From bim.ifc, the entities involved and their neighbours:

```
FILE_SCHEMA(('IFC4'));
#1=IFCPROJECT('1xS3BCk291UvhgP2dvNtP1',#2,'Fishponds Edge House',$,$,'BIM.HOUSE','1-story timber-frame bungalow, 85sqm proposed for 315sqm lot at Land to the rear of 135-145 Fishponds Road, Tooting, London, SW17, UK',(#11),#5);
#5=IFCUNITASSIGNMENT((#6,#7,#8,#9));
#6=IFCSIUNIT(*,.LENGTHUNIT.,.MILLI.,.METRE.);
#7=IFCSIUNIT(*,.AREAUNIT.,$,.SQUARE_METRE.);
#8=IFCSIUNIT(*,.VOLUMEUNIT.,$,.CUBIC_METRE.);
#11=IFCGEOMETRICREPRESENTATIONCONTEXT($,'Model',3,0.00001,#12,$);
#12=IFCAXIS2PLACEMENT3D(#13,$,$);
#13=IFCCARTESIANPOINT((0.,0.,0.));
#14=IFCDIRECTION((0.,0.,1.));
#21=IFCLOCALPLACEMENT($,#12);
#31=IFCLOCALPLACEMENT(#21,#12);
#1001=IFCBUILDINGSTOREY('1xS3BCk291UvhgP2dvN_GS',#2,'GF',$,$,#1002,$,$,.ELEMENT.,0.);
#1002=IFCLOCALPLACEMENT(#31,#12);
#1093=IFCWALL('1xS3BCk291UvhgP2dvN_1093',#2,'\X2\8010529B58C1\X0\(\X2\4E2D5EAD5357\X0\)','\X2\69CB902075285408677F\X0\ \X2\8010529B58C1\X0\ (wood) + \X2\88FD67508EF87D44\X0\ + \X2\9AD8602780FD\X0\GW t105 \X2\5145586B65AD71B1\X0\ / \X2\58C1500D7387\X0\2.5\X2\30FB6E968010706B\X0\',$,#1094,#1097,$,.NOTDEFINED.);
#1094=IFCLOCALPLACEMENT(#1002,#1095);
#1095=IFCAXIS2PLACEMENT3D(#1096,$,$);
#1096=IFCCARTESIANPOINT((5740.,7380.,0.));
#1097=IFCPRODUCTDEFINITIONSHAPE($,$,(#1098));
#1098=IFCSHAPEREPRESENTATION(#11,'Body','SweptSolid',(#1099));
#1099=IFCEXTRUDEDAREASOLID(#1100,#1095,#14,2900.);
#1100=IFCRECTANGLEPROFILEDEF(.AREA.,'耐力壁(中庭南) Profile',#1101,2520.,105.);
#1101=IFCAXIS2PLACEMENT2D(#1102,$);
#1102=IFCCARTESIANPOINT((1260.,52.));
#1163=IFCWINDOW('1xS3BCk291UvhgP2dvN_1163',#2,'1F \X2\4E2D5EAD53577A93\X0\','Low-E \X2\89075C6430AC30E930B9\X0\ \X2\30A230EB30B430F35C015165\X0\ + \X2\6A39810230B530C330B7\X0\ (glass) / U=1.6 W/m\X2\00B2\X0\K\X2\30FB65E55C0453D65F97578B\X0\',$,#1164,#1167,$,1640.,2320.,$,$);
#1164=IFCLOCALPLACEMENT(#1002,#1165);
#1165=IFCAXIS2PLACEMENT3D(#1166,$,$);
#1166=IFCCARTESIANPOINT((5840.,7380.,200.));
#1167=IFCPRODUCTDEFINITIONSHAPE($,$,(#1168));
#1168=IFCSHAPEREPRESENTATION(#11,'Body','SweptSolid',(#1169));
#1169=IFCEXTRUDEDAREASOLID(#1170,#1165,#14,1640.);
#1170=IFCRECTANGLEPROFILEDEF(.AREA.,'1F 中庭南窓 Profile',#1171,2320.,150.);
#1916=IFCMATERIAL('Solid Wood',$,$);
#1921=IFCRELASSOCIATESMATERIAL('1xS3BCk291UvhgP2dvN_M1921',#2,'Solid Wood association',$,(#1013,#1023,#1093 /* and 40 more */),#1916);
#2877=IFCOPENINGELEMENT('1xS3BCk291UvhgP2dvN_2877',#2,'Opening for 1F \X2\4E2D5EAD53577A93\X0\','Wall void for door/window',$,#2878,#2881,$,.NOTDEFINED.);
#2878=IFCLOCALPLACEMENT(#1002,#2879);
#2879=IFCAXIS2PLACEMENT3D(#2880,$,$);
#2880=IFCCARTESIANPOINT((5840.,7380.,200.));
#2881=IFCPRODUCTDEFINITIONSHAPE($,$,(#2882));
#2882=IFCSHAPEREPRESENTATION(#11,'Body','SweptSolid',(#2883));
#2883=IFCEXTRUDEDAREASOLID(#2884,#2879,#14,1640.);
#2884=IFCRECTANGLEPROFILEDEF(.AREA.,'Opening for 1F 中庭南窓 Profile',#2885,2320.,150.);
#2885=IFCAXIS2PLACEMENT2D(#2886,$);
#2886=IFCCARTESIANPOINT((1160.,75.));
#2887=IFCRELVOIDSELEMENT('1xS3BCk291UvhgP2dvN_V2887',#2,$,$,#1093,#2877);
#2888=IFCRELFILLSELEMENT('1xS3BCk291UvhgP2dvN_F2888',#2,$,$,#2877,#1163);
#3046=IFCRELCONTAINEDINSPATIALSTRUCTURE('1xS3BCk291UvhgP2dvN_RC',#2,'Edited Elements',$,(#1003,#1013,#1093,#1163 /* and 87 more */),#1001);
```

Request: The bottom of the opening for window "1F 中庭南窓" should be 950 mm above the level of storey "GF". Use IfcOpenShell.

```python
import numpy as np
import ifcopenshell
import ifcopenshell.api.geometry
import ifcopenshell.geom
import ifcopenshell.util.element
import ifcopenshell.util.placement
import ifcopenshell.util.shape
import ifcopenshell.util.unit

model = ifcopenshell.open("bim.ifc")
unit_scale = ifcopenshell.util.unit.calculate_unit_scale(model)

window = model.by_guid("1xS3BCk291UvhgP2dvN_1163")
opening = window.FillsVoids[0].RelatingOpeningElement
storey = ifcopenshell.util.element.get_container(window, ifc_class="IfcBuildingStorey")
level = ifcopenshell.util.placement.get_local_placement(storey.ObjectPlacement)[2, 3]

# The opening's origin need not be at the sill, so measure its lowest point.
shape = ifcopenshell.geom.create_shape(ifcopenshell.geom.settings(), opening)
bottom = ifcopenshell.util.shape.get_shape_bottom_elevation(shape, shape.geometry) / unit_scale
dz = level + 950.0 - bottom

shift = np.array([0.0, 0.0, dz])
# The window is not placed relative to its opening, so move both.
for product in (opening, window):
    matrix = ifcopenshell.util.placement.get_local_placement(product.ObjectPlacement)
    matrix[:3, 3] += shift
    ifcopenshell.api.geometry.edit_object_placement(model, product=product, matrix=matrix, is_si=False)

print(f"moved by {dz * unit_scale:+.3f} m")

model.write("bim_rev.ifc")
```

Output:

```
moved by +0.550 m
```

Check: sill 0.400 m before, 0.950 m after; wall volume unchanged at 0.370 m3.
